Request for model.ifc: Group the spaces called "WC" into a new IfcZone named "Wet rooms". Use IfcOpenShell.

First a look at what the model holds.

```python
import ifcopenshell

model = ifcopenshell.open("model.ifc")
print(model.schema)
seen = {}
for space in model.by_type("IfcSpace"):
    seen[space.LongName] = seen.get(space.LongName, 0) + 1
for name, count in sorted(seen.items(), key=str):
    print(count, "x", name)
print("zones:", [z.Name for z in model.by_type("IfcZone")][:20])
```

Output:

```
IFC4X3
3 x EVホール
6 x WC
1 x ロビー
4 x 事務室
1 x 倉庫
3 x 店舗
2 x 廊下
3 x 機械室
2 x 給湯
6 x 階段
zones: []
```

```python
import ifcopenshell
import ifcopenshell.api.group
import ifcopenshell.api.root

model = ifcopenshell.open("model.ifc")

names = {"WC"}
spaces = [s for s in model.by_type("IfcSpace") if s.LongName in names]

zone = ifcopenshell.api.root.create_entity(model, ifc_class="IfcZone", name="Wet rooms")
ifcopenshell.api.group.assign_group(model, products=spaces, group=zone)
print(len(spaces), "spaces in", zone.Name)

model.write("model_updated.ifc")
```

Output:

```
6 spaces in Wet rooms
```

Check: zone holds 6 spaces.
